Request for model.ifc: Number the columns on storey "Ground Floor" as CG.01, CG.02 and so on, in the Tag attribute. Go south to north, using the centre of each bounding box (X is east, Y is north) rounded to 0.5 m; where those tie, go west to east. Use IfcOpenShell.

First a look at what the model holds.

```python
import ifcopenshell
import ifcopenshell.util.element
import ifcopenshell.util.placement

model = ifcopenshell.open("model.ifc")
print(model.schema)
storey = next(s for s in model.by_type("IfcBuildingStorey") if s.Name == "Ground Floor")
columns = [e for e in ifcopenshell.util.element.get_decomposition(storey) if e.is_a("IfcColumn")]
for e in sorted(columns, key=lambda e: e.id()):
    origin = ifcopenshell.util.placement.get_local_placement(e.ObjectPlacement)[:3, 3]
    print(e.id(), e.Tag, e.Name, origin.round(2) + 0.0, sep=" | ")
```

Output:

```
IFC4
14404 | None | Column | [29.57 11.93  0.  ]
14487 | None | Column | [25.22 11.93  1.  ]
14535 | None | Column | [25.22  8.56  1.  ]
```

```python
import ifcopenshell
import ifcopenshell.geom
import ifcopenshell.util.element
import ifcopenshell.util.shape

model = ifcopenshell.open("model.ifc")
settings = ifcopenshell.geom.settings()
settings.set("use-world-coords", True)


def centre(element):
    shape = ifcopenshell.geom.create_shape(settings, element)
    return ifcopenshell.util.shape.get_bbox_centroid(shape.geometry)


storey = next(s for s in model.by_type("IfcBuildingStorey") if s.Name == "Ground Floor")
columns = [e for e in ifcopenshell.util.element.get_decomposition(storey) if e.is_a("IfcColumn")]

# Insertion points can sit at a corner or the storey origin, so sort by the geometry (in metres).
centres = {e: centre(e) for e in columns}
columns.sort(key=lambda e: (round(centres[e][1] / 0.5), centres[e][0]))

for i, e in enumerate(columns, start=1):
    number = f"CG.{i:02d}"
    e.Tag = number
    print(e.id(), number)

model.write("model_rev.ifc")
```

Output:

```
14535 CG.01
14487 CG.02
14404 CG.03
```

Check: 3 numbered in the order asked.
